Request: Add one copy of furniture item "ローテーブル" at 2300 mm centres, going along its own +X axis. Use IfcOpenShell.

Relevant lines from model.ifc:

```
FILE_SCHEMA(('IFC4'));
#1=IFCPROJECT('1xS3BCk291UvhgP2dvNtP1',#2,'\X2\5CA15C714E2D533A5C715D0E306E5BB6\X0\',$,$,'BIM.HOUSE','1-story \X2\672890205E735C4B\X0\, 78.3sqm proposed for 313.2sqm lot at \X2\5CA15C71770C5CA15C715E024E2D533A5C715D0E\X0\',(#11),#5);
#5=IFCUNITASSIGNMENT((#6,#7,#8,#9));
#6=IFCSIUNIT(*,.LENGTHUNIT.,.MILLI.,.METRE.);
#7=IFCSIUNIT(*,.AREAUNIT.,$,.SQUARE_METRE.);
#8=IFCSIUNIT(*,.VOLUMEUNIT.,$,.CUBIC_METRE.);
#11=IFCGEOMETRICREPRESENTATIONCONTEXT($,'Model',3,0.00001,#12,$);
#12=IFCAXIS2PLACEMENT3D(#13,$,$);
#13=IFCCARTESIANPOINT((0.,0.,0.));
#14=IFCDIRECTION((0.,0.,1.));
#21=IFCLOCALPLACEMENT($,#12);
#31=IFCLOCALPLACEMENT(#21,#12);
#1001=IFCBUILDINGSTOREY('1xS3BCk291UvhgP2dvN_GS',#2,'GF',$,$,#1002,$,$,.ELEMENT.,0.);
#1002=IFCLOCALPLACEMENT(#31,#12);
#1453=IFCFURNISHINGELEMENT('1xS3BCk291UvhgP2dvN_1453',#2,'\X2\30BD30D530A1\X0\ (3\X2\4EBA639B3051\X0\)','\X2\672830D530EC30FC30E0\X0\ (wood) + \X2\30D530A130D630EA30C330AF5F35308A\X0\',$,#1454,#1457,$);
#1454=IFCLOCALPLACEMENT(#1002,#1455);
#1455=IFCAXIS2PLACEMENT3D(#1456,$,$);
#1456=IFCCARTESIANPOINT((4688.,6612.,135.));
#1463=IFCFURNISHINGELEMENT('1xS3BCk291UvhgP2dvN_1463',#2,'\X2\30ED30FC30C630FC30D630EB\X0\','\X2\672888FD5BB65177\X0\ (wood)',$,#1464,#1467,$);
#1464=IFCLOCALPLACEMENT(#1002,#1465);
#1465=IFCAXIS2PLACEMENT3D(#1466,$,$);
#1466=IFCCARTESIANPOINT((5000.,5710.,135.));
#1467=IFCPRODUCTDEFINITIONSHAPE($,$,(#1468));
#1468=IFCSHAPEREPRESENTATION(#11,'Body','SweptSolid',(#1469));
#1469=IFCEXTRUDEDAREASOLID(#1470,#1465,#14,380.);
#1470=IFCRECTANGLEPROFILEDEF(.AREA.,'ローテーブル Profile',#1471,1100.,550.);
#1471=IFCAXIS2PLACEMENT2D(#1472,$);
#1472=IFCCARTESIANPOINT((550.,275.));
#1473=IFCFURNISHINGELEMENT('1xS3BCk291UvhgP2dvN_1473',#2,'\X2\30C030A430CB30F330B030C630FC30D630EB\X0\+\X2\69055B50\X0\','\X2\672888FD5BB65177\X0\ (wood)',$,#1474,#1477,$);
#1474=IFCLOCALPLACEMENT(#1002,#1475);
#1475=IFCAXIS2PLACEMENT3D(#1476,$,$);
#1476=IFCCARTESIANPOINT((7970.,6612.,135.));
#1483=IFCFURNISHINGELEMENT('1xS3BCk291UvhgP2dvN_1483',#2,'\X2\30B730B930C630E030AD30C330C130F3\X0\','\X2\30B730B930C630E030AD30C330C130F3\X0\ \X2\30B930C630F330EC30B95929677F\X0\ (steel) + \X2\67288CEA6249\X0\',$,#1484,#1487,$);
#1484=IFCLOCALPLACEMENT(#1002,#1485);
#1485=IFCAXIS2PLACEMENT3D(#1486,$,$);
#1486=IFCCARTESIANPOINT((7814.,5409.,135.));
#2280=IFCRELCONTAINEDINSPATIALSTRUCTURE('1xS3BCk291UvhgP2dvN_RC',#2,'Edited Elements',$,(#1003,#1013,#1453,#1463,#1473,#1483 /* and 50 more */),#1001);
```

```python
import ifcopenshell
import ifcopenshell.api.geometry
import ifcopenshell.api.root
import ifcopenshell.util.element
import ifcopenshell.util.placement
import ifcopenshell.util.unit

model = ifcopenshell.open("model.ifc")
unit_scale = ifcopenshell.util.unit.calculate_unit_scale(model)


def reuse_history(source, copy):
    """copy_class also copies each property set's owner history, people and application; keep the originals."""
    for rel in copy.IsDefinedBy:
        if rel.is_a("IfcRelDefinesByProperties") and (history := rel.RelatingPropertyDefinition.OwnerHistory):
            rel.RelatingPropertyDefinition.OwnerHistory = source.OwnerHistory
            ifcopenshell.util.element.remove_deep2(model, history)


source = model.by_id(1463)
base = ifcopenshell.util.placement.get_local_placement(source.ObjectPlacement)
step = base[:3, 0] * 2.3 / unit_scale

for i in range(1, 2):
    copy = ifcopenshell.api.root.copy_class(model, product=source)
    copy.Representation = ifcopenshell.util.element.copy_deep(
        model, source.Representation, exclude=["IfcGeometricRepresentationContext", "IfcRepresentationMap"]
    )
    reuse_history(source, copy)
    matrix = base.copy()
    matrix[:3, 3] += i * step
    print("added at", matrix[:3, 3].round(3) + 0.0)
    ifcopenshell.api.geometry.edit_object_placement(model, product=copy, matrix=matrix, is_si=False)

model.write("model_rev.ifc")
```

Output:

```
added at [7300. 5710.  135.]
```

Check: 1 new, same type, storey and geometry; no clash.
